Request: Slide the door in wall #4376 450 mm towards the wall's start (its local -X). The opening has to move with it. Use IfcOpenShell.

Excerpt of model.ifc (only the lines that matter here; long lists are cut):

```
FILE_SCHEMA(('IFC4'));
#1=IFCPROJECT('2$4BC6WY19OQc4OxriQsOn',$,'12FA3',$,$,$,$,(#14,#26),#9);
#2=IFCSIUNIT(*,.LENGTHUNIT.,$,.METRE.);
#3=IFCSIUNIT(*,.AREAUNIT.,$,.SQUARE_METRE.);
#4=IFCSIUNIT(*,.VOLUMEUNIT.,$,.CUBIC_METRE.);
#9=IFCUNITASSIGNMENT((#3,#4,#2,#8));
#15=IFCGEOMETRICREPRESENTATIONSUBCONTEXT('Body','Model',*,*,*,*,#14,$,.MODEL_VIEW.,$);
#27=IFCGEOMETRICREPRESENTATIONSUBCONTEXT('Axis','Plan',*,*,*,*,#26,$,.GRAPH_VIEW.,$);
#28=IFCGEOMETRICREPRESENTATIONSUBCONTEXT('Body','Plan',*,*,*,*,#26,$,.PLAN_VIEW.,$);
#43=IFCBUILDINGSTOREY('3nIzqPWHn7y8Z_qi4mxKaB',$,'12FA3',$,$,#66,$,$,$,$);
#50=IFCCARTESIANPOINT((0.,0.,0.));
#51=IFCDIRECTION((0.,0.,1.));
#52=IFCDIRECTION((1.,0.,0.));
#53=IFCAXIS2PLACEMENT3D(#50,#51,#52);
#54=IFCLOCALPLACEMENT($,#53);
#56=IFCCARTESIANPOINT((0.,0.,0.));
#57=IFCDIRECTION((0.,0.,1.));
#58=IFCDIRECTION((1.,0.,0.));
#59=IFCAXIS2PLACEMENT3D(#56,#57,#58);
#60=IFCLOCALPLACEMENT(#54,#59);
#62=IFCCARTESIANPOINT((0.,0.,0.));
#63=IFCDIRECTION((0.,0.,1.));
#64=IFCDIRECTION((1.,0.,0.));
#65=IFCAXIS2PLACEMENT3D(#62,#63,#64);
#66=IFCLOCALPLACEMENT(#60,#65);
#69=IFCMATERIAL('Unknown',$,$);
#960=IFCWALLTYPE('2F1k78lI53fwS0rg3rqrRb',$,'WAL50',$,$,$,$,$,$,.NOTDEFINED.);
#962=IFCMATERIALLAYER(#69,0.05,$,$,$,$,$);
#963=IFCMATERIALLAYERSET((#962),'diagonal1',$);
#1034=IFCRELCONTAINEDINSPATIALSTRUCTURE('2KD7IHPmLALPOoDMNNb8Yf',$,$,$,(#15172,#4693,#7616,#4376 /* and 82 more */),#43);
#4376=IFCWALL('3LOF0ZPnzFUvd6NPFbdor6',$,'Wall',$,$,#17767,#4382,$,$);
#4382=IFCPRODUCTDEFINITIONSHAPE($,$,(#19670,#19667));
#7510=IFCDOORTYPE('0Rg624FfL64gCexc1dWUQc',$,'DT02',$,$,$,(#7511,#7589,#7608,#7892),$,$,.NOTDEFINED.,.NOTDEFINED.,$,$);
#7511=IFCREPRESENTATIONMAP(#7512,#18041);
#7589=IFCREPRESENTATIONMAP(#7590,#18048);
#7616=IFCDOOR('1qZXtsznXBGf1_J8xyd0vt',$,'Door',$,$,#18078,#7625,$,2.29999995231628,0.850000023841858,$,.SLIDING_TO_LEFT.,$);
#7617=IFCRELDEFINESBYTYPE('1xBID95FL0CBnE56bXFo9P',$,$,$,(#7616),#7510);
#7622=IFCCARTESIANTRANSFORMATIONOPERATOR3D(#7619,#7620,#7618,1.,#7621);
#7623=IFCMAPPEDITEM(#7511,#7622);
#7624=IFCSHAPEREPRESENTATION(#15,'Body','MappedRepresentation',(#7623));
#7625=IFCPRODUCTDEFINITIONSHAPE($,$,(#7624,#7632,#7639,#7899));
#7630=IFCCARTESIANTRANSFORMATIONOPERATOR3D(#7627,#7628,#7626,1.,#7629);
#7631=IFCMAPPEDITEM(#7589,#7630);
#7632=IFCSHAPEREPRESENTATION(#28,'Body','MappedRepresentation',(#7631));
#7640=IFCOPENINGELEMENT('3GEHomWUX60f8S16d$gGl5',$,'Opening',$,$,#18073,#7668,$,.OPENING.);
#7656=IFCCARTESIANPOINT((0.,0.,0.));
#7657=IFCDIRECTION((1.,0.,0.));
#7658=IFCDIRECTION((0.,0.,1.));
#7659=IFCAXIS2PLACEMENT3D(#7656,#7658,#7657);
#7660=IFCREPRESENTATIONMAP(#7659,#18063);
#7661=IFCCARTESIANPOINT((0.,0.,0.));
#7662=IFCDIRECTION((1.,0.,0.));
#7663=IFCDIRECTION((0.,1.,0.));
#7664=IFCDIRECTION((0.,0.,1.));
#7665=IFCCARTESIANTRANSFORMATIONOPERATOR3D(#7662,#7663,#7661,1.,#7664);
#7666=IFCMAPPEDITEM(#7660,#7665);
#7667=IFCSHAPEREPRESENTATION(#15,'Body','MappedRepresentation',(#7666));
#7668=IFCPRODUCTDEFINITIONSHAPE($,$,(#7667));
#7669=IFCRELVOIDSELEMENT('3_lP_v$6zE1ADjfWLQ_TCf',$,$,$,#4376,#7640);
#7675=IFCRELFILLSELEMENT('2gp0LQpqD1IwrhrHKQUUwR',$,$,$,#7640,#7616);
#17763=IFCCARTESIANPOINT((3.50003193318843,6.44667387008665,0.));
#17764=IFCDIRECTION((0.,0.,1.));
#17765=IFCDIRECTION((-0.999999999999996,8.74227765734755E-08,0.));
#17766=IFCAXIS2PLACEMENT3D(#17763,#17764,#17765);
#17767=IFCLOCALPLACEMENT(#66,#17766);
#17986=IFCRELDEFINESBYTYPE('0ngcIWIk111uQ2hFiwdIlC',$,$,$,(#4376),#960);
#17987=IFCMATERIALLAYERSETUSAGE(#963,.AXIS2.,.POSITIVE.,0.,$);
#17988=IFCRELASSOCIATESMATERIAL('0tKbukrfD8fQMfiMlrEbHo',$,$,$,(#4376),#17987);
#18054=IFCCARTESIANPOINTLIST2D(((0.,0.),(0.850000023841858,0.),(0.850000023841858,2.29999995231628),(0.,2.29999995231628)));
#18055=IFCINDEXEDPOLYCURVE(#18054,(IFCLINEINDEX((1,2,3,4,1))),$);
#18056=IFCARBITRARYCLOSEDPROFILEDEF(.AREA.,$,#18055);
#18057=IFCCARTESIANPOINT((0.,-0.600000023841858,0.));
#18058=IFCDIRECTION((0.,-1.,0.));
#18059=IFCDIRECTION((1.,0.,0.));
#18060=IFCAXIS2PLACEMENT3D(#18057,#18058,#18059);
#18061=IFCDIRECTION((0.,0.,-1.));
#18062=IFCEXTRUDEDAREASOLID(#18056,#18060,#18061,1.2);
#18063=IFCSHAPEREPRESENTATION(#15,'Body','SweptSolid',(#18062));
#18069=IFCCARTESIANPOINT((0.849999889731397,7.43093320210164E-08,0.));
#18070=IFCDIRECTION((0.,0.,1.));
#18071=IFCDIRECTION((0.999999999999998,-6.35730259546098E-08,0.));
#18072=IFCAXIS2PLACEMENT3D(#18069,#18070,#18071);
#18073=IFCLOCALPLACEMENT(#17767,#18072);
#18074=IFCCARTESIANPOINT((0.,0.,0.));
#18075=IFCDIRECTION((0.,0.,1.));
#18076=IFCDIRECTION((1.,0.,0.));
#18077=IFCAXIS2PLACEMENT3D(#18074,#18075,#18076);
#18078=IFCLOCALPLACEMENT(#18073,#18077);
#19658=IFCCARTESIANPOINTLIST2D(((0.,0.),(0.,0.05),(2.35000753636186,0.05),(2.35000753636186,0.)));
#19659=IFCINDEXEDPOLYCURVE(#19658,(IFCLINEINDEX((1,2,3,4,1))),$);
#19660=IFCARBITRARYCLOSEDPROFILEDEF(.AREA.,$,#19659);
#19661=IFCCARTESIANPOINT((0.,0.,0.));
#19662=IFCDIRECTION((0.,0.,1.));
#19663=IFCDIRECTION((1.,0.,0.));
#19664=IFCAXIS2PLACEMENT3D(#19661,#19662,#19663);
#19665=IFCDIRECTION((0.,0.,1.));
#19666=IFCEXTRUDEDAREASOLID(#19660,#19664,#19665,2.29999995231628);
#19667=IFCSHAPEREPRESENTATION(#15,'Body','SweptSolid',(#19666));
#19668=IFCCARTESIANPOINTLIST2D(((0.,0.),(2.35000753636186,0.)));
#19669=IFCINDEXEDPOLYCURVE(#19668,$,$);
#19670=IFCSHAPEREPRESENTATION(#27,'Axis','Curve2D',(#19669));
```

```python
import ifcopenshell
import ifcopenshell.api.geometry
import ifcopenshell.util.placement
import ifcopenshell.util.unit

model = ifcopenshell.open("model.ifc")
unit_scale = ifcopenshell.util.unit.calculate_unit_scale(model)

door = model.by_id(7616)
opening = door.FillsVoids[0].RelatingOpeningElement
wall = opening.VoidsElements[0].RelatingBuildingElement

wall_matrix = ifcopenshell.util.placement.get_local_placement(wall.ObjectPlacement)
shift = wall_matrix[:3, 0] * -0.45 / unit_scale
before = ifcopenshell.util.placement.get_local_placement(door.ObjectPlacement)[:3, 3].copy()

# The door is placed relative to its opening, so it follows when the opening moves.
matrix = ifcopenshell.util.placement.get_local_placement(opening.ObjectPlacement)
matrix[:3, 3] += shift
ifcopenshell.api.geometry.edit_object_placement(
    model, product=opening, matrix=matrix, is_si=False, should_transform_children=True
)

after = ifcopenshell.util.placement.get_local_placement(door.ObjectPlacement)[:3, 3]
print("door moved by", (after - before).round(3) + 0.0)

model.write("model_rev.ifc")
```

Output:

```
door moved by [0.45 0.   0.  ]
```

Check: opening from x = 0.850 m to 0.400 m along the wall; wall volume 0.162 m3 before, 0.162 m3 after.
